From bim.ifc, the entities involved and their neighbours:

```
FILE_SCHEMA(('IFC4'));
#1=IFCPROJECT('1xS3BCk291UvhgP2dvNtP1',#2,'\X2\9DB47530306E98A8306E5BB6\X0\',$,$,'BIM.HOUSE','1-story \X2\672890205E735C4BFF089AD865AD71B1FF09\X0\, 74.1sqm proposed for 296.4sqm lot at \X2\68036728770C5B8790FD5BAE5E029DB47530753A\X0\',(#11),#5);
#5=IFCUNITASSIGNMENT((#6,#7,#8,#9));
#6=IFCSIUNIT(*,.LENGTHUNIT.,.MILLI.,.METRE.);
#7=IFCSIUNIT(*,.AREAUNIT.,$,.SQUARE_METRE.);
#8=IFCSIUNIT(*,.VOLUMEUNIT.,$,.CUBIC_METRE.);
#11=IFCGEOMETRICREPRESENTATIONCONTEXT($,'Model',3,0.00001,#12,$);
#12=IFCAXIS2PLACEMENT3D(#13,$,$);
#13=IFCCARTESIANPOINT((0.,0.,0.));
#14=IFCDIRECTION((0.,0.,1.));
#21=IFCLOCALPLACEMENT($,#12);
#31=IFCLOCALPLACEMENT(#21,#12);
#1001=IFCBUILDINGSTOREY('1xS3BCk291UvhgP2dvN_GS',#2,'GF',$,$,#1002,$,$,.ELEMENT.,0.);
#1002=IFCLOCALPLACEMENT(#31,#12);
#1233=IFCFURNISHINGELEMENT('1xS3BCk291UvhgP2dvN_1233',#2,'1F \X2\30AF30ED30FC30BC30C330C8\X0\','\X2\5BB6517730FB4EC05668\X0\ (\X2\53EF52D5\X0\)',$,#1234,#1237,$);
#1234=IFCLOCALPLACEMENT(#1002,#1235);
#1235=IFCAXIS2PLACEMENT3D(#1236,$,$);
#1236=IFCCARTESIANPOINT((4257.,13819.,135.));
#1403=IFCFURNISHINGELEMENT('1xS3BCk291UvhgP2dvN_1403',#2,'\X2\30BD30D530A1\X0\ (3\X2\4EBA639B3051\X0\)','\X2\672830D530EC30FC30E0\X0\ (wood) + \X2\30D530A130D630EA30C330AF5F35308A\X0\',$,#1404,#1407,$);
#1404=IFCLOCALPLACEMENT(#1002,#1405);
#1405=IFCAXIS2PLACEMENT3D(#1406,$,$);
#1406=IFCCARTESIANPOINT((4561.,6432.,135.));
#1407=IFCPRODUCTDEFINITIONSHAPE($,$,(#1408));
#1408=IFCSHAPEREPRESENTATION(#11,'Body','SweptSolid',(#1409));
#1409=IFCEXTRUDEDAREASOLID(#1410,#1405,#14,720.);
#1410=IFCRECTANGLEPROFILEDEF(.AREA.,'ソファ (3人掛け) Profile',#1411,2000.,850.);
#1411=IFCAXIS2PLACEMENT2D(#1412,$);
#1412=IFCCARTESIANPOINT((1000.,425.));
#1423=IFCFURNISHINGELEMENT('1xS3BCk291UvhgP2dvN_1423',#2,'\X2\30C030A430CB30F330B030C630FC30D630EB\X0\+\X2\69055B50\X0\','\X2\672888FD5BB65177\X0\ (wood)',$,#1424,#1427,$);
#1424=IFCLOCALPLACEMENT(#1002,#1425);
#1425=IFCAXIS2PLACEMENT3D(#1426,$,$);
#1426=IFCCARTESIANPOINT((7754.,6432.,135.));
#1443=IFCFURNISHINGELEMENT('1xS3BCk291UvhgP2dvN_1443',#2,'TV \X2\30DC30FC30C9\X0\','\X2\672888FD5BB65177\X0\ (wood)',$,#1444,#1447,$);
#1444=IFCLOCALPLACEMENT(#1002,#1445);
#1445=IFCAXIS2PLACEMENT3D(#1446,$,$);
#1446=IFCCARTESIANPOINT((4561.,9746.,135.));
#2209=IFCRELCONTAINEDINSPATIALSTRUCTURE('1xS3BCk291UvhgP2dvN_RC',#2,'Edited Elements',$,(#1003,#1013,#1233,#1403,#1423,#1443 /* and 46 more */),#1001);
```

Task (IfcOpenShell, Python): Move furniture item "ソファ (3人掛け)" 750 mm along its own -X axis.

```python
import ifcopenshell
import ifcopenshell.api.geometry
import ifcopenshell.util.placement

model = ifcopenshell.open("bim.ifc")

item = model.by_guid("1xS3BCk291UvhgP2dvN_1403")
matrix = ifcopenshell.util.placement.get_local_placement(item.ObjectPlacement)
matrix[:3, 3] -= matrix[:3, 0] * 750.0
ifcopenshell.api.geometry.edit_object_placement(model, product=item, matrix=matrix, is_si=False)

print(ifcopenshell.util.placement.get_local_placement(item.ObjectPlacement).round(3) + 0.0)

model.write("bim_rev.ifc")
```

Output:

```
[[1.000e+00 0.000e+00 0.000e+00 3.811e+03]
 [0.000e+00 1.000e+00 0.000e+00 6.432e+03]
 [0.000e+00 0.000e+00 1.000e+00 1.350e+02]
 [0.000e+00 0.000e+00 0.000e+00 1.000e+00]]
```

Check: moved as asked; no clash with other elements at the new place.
